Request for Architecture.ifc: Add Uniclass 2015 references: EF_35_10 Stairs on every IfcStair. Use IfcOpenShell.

First a look at what the model holds.

```python
import ifcopenshell

model = ifcopenshell.open("Architecture.ifc")
print(model.schema)
print("classifications:", [c.Name for c in model.by_type("IfcClassification")])
for ifc_class in ("IfcDoor", "IfcRoof", "IfcStair", "IfcWall", "IfcWindow"):
    print(ifc_class, len(model.by_type(ifc_class)))
```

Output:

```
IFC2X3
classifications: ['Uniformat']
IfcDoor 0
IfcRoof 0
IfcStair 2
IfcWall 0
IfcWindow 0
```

```python
import ifcopenshell
import ifcopenshell.api.classification

model = ifcopenshell.open("Architecture.ifc")

# IFC2X3 requires Source and Edition and has no link from the project to the system.
system = model.create_entity("IfcClassification", Source="NBS", Edition="2015", Name="Uniclass 2015")

codes = {
    "IfcStair": ("EF_35_10", "Stairs"),
}
for ifc_class, (code, name) in codes.items():
    products = model.by_type(ifc_class)
    ifcopenshell.api.classification.add_reference(
        model, products=products, classification=system, identification=code, name=name
    )
    print(code, len(products))

model.write("Architecture-out.ifc")
```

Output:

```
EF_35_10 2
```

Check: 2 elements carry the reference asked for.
